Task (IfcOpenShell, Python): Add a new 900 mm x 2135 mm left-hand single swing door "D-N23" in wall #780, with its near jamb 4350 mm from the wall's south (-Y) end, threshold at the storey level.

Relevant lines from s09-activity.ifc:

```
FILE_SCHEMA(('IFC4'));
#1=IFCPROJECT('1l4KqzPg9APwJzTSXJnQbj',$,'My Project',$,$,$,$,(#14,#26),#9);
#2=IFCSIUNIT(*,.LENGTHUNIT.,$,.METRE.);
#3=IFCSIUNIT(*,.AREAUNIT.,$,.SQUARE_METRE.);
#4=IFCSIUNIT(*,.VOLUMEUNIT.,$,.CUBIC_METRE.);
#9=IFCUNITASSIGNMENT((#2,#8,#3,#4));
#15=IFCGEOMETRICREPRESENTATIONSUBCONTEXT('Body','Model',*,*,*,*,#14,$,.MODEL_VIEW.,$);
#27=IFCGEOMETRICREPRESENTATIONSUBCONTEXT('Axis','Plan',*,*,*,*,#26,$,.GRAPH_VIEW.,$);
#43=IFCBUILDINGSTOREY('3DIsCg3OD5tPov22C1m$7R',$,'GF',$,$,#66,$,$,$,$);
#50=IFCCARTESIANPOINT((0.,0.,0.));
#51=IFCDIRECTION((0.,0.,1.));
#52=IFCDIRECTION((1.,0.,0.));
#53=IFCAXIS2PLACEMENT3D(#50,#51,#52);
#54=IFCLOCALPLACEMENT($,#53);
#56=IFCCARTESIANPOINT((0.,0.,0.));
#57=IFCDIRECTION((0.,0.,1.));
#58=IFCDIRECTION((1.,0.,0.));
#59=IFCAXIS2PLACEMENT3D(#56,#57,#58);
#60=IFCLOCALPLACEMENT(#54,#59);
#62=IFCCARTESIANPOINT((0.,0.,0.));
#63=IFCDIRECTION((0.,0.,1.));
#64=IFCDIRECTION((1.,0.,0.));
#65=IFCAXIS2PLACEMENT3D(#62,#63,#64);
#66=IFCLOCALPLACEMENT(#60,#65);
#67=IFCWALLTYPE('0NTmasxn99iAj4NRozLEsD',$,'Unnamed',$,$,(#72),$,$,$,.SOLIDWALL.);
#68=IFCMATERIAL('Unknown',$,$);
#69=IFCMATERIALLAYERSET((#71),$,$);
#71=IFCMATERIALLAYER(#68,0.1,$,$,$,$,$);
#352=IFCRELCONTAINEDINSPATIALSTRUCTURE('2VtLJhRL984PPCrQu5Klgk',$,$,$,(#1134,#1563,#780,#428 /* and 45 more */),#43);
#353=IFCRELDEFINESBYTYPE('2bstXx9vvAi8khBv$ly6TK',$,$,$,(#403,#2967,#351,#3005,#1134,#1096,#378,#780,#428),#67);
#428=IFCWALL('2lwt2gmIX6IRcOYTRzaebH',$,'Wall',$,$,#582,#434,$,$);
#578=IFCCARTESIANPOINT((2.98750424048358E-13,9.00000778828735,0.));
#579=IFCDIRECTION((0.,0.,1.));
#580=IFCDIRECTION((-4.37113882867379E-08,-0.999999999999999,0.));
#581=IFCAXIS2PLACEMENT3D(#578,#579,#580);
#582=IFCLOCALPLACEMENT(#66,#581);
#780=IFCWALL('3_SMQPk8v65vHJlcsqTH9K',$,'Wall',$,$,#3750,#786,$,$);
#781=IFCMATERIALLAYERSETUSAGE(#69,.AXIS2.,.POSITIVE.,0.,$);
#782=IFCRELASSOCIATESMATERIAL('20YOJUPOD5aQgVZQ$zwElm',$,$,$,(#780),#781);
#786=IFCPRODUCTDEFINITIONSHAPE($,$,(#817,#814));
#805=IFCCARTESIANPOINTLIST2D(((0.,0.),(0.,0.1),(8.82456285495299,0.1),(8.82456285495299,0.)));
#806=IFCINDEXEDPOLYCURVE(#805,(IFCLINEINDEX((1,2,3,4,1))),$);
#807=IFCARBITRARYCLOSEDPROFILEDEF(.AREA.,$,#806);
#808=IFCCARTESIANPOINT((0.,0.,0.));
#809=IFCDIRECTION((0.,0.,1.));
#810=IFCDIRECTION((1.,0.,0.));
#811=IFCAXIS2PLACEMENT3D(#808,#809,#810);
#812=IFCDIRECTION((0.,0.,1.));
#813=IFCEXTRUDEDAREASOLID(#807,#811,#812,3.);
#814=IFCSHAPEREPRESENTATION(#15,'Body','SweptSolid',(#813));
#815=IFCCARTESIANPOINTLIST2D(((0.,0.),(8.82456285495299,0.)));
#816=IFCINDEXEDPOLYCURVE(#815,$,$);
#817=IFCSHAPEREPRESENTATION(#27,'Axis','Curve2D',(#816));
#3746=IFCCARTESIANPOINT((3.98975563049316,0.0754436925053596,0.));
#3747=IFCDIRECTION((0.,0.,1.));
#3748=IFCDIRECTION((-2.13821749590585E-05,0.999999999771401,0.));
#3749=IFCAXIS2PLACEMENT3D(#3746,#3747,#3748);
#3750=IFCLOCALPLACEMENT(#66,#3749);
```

```python
import numpy as np
import ifcopenshell
import ifcopenshell.api.feature
import ifcopenshell.api.geometry
import ifcopenshell.api.root
import ifcopenshell.api.spatial
import ifcopenshell.geom
import ifcopenshell.util.element
import ifcopenshell.util.placement
import ifcopenshell.util.representation
import ifcopenshell.util.shape
import ifcopenshell.util.unit

model = ifcopenshell.open("s09-activity.ifc")
unit_scale = ifcopenshell.util.unit.calculate_unit_scale(model)
settings = ifcopenshell.geom.settings()


def volume(element):
    """Net volume in cubic metres, openings subtracted."""
    shape = ifcopenshell.geom.create_shape(settings, element)
    return ifcopenshell.util.shape.get_volume(shape.geometry)


wall = model.by_id(780)
storey = ifcopenshell.util.element.get_container(wall, ifc_class="IfcBuildingStorey")
context = ifcopenshell.util.representation.get_context(model, "Model", "Body", "MODEL_VIEW")
before = volume(wall)

width, height, from_end, sill = 0.9, 2.135, 4.35, 0.0  # metres

# The wall runs along its own X axis, and the end named is its -X end.
wall_shape = ifcopenshell.geom.create_shape(settings, wall)
x, y, z = ifcopenshell.util.shape.get_vertices(wall_shape.geometry).T
start = x.min() + from_end
face, thickness = float(y.min()), float(y.max() - y.min())
wall_matrix = ifcopenshell.util.placement.get_local_placement(wall.ObjectPlacement)
level = ifcopenshell.util.placement.get_local_placement(storey.ObjectPlacement)[2, 3]


def in_wall(x, y):
    """Placement at x, y metres in the wall's axes, at sill height."""
    matrix = wall_matrix.copy()
    matrix[:, 3] = wall_matrix @ np.array([x / unit_scale, y / unit_scale, 0.0, 1.0])
    matrix[2, 3] = level + sill / unit_scale
    return matrix


# Opening: a box that overshoots both wall faces by 50 mm.
opening = ifcopenshell.api.root.create_entity(model, ifc_class="IfcOpeningElement", predefined_type="OPENING")
box = ifcopenshell.api.geometry.add_wall_representation(
    model, context=context, length=width, height=height, thickness=thickness + 0.1
)
ifcopenshell.api.geometry.assign_representation(model, product=opening, representation=box)
ifcopenshell.api.geometry.edit_object_placement(model, product=opening, matrix=in_wall(start, face - 0.05), is_si=False)
ifcopenshell.api.feature.add_feature(model, feature=opening, element=wall)

door = ifcopenshell.api.root.create_entity(model, ifc_class="IfcDoor", name="D-N23", predefined_type="DOOR")
door.OverallWidth, door.OverallHeight = width / unit_scale, height / unit_scale
door.OperationType = "SINGLE_SWING_LEFT"
body = ifcopenshell.api.geometry.add_door_representation(
    model,
    context=context,
    overall_width=door.OverallWidth,
    overall_height=door.OverallHeight,
    operation_type="SINGLE_SWING_LEFT",
    lining_properties={"LiningDepth": thickness / unit_scale, "ThresholdDepth": thickness / unit_scale},
)
ifcopenshell.api.geometry.assign_representation(model, product=door, representation=body)
ifcopenshell.api.spatial.assign_container(model, products=[door], relating_structure=storey)
ifcopenshell.api.feature.add_filling(model, opening=opening, element=door)

# The lining spans the wall, so the door starts at the wall face.
ifcopenshell.api.geometry.edit_object_placement(model, product=door, matrix=in_wall(start, face), is_si=False)

after = volume(wall)

print(f"wall volume {before:.3f} -> {after:.3f} m3")

model.write("s09-activity-out.ifc")
```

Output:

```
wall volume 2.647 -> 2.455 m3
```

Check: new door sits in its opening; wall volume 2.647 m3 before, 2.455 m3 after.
